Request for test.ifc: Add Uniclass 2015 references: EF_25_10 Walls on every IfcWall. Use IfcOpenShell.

First a look at what the model holds.

```python
import ifcopenshell

model = ifcopenshell.open("test.ifc")
print(model.schema)
print("classifications:", [c.Name for c in model.by_type("IfcClassification")])
for ifc_class in ("IfcDoor", "IfcRoof", "IfcStair", "IfcWall", "IfcWindow"):
    print(ifc_class, len(model.by_type(ifc_class)))
```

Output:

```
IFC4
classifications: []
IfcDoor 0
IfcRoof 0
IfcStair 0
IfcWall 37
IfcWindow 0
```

```python
import ifcopenshell
import ifcopenshell.api.classification

model = ifcopenshell.open("test.ifc")

system = ifcopenshell.api.classification.add_classification(model, classification="Uniclass 2015")

codes = {
    "IfcWall": ("EF_25_10", "Walls"),
}
for ifc_class, (code, name) in codes.items():
    products = model.by_type(ifc_class)
    ifcopenshell.api.classification.add_reference(
        model, products=products, classification=system, identification=code, name=name
    )
    print(code, len(products))

model.write("test_v2.ifc")
```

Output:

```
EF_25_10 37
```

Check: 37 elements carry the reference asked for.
